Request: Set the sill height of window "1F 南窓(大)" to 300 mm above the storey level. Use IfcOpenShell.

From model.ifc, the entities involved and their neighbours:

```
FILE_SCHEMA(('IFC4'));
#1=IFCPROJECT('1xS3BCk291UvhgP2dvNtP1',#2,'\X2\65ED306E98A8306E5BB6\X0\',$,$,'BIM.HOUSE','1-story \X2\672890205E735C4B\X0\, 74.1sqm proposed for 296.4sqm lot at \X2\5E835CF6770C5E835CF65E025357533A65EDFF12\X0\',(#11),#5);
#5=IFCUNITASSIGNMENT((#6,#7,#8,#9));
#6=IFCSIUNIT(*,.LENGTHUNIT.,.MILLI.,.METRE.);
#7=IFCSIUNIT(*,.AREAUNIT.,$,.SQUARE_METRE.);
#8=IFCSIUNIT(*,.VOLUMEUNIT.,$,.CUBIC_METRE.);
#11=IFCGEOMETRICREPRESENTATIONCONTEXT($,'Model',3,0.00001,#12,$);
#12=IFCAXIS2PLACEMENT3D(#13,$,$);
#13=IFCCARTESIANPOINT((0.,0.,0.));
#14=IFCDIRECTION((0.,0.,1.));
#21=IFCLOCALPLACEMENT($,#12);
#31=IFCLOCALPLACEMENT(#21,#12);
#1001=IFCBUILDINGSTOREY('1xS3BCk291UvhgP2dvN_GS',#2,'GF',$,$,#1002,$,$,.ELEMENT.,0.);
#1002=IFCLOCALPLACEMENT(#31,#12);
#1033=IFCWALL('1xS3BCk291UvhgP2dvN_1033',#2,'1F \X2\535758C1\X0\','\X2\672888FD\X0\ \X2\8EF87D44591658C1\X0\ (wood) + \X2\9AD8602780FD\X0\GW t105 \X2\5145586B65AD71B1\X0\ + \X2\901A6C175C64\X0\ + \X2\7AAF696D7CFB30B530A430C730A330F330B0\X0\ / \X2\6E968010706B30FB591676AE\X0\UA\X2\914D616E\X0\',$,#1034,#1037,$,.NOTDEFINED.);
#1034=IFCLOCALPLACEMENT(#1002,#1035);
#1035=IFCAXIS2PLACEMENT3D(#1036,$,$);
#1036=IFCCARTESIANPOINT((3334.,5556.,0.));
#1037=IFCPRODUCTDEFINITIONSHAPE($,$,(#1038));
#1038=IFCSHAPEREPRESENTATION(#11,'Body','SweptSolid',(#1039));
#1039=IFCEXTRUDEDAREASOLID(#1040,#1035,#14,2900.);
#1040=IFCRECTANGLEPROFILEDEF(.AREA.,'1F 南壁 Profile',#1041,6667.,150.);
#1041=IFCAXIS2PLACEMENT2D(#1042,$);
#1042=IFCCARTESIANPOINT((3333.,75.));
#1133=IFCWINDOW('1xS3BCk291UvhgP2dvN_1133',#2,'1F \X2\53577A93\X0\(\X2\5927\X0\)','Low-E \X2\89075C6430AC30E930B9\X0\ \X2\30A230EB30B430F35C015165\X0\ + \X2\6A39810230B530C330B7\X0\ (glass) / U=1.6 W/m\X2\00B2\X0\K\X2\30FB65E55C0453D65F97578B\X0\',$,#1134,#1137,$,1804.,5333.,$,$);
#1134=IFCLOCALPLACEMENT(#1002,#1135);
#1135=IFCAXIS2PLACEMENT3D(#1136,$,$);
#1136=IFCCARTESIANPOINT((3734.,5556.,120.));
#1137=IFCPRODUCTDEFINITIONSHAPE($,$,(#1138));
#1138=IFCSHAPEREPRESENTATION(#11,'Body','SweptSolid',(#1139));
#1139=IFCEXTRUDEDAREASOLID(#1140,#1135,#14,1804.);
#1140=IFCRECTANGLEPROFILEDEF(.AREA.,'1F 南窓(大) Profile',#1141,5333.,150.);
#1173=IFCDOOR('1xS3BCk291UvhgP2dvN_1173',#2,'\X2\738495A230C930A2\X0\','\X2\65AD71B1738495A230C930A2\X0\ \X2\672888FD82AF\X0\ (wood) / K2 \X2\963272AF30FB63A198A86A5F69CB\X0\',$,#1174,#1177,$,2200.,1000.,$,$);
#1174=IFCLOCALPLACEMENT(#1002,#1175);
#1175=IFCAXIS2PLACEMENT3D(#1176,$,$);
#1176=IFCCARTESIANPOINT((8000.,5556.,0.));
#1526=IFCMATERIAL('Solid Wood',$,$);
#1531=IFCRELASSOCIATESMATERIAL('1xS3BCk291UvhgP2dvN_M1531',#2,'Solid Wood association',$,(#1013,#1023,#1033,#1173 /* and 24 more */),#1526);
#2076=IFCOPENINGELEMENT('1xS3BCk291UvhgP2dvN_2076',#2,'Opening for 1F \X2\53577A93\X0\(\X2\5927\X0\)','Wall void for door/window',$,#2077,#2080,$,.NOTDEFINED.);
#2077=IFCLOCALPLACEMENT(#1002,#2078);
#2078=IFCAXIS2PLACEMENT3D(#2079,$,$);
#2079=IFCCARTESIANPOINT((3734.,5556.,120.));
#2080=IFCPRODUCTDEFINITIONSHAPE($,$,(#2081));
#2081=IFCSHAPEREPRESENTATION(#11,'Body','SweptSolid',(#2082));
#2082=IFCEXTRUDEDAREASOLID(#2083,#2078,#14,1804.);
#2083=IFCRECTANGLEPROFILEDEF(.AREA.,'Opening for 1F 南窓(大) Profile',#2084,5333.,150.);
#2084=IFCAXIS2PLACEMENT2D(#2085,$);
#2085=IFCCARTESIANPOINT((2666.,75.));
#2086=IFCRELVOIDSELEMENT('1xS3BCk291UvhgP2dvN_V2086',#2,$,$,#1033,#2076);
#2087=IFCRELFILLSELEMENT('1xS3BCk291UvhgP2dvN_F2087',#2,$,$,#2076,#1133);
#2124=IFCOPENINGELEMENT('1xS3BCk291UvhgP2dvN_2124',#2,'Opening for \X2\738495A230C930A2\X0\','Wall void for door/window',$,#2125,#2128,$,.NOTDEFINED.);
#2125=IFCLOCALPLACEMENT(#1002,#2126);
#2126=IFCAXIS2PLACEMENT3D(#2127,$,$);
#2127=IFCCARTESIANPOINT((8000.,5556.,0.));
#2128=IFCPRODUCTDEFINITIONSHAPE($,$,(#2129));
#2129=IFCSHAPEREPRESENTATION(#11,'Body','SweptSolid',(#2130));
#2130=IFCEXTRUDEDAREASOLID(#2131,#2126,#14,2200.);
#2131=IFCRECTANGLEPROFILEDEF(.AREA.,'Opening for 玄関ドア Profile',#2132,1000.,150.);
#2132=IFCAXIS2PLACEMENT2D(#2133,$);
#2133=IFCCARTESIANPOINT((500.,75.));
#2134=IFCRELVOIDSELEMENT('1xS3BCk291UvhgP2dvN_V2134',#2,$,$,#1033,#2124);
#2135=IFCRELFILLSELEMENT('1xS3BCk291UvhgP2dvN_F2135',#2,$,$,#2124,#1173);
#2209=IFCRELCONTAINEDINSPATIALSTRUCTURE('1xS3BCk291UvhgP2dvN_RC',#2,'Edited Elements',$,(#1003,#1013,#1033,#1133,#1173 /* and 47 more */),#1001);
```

```python
import numpy as np
import ifcopenshell
import ifcopenshell.api.geometry
import ifcopenshell.geom
import ifcopenshell.util.element
import ifcopenshell.util.placement
import ifcopenshell.util.shape
import ifcopenshell.util.unit

model = ifcopenshell.open("model.ifc")
unit_scale = ifcopenshell.util.unit.calculate_unit_scale(model)

window = model.by_guid("1xS3BCk291UvhgP2dvN_1133")
opening = window.FillsVoids[0].RelatingOpeningElement
storey = ifcopenshell.util.element.get_container(window, ifc_class="IfcBuildingStorey")
level = ifcopenshell.util.placement.get_local_placement(storey.ObjectPlacement)[2, 3]

# The opening's origin need not be at the sill, so measure its lowest point.
shape = ifcopenshell.geom.create_shape(ifcopenshell.geom.settings(), opening)
bottom = ifcopenshell.util.shape.get_shape_bottom_elevation(shape, shape.geometry) / unit_scale
dz = level + 0.3 / unit_scale - bottom

shift = np.array([0.0, 0.0, dz])
# The window is not placed relative to its opening, so move both.
for product in (opening, window):
    matrix = ifcopenshell.util.placement.get_local_placement(product.ObjectPlacement)
    matrix[:3, 3] += shift
    ifcopenshell.api.geometry.edit_object_placement(model, product=product, matrix=matrix, is_si=False)

print(f"moved by {dz * unit_scale:+.3f} m")

model.write("model_edited.ifc")
```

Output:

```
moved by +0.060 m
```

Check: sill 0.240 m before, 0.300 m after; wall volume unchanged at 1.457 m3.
